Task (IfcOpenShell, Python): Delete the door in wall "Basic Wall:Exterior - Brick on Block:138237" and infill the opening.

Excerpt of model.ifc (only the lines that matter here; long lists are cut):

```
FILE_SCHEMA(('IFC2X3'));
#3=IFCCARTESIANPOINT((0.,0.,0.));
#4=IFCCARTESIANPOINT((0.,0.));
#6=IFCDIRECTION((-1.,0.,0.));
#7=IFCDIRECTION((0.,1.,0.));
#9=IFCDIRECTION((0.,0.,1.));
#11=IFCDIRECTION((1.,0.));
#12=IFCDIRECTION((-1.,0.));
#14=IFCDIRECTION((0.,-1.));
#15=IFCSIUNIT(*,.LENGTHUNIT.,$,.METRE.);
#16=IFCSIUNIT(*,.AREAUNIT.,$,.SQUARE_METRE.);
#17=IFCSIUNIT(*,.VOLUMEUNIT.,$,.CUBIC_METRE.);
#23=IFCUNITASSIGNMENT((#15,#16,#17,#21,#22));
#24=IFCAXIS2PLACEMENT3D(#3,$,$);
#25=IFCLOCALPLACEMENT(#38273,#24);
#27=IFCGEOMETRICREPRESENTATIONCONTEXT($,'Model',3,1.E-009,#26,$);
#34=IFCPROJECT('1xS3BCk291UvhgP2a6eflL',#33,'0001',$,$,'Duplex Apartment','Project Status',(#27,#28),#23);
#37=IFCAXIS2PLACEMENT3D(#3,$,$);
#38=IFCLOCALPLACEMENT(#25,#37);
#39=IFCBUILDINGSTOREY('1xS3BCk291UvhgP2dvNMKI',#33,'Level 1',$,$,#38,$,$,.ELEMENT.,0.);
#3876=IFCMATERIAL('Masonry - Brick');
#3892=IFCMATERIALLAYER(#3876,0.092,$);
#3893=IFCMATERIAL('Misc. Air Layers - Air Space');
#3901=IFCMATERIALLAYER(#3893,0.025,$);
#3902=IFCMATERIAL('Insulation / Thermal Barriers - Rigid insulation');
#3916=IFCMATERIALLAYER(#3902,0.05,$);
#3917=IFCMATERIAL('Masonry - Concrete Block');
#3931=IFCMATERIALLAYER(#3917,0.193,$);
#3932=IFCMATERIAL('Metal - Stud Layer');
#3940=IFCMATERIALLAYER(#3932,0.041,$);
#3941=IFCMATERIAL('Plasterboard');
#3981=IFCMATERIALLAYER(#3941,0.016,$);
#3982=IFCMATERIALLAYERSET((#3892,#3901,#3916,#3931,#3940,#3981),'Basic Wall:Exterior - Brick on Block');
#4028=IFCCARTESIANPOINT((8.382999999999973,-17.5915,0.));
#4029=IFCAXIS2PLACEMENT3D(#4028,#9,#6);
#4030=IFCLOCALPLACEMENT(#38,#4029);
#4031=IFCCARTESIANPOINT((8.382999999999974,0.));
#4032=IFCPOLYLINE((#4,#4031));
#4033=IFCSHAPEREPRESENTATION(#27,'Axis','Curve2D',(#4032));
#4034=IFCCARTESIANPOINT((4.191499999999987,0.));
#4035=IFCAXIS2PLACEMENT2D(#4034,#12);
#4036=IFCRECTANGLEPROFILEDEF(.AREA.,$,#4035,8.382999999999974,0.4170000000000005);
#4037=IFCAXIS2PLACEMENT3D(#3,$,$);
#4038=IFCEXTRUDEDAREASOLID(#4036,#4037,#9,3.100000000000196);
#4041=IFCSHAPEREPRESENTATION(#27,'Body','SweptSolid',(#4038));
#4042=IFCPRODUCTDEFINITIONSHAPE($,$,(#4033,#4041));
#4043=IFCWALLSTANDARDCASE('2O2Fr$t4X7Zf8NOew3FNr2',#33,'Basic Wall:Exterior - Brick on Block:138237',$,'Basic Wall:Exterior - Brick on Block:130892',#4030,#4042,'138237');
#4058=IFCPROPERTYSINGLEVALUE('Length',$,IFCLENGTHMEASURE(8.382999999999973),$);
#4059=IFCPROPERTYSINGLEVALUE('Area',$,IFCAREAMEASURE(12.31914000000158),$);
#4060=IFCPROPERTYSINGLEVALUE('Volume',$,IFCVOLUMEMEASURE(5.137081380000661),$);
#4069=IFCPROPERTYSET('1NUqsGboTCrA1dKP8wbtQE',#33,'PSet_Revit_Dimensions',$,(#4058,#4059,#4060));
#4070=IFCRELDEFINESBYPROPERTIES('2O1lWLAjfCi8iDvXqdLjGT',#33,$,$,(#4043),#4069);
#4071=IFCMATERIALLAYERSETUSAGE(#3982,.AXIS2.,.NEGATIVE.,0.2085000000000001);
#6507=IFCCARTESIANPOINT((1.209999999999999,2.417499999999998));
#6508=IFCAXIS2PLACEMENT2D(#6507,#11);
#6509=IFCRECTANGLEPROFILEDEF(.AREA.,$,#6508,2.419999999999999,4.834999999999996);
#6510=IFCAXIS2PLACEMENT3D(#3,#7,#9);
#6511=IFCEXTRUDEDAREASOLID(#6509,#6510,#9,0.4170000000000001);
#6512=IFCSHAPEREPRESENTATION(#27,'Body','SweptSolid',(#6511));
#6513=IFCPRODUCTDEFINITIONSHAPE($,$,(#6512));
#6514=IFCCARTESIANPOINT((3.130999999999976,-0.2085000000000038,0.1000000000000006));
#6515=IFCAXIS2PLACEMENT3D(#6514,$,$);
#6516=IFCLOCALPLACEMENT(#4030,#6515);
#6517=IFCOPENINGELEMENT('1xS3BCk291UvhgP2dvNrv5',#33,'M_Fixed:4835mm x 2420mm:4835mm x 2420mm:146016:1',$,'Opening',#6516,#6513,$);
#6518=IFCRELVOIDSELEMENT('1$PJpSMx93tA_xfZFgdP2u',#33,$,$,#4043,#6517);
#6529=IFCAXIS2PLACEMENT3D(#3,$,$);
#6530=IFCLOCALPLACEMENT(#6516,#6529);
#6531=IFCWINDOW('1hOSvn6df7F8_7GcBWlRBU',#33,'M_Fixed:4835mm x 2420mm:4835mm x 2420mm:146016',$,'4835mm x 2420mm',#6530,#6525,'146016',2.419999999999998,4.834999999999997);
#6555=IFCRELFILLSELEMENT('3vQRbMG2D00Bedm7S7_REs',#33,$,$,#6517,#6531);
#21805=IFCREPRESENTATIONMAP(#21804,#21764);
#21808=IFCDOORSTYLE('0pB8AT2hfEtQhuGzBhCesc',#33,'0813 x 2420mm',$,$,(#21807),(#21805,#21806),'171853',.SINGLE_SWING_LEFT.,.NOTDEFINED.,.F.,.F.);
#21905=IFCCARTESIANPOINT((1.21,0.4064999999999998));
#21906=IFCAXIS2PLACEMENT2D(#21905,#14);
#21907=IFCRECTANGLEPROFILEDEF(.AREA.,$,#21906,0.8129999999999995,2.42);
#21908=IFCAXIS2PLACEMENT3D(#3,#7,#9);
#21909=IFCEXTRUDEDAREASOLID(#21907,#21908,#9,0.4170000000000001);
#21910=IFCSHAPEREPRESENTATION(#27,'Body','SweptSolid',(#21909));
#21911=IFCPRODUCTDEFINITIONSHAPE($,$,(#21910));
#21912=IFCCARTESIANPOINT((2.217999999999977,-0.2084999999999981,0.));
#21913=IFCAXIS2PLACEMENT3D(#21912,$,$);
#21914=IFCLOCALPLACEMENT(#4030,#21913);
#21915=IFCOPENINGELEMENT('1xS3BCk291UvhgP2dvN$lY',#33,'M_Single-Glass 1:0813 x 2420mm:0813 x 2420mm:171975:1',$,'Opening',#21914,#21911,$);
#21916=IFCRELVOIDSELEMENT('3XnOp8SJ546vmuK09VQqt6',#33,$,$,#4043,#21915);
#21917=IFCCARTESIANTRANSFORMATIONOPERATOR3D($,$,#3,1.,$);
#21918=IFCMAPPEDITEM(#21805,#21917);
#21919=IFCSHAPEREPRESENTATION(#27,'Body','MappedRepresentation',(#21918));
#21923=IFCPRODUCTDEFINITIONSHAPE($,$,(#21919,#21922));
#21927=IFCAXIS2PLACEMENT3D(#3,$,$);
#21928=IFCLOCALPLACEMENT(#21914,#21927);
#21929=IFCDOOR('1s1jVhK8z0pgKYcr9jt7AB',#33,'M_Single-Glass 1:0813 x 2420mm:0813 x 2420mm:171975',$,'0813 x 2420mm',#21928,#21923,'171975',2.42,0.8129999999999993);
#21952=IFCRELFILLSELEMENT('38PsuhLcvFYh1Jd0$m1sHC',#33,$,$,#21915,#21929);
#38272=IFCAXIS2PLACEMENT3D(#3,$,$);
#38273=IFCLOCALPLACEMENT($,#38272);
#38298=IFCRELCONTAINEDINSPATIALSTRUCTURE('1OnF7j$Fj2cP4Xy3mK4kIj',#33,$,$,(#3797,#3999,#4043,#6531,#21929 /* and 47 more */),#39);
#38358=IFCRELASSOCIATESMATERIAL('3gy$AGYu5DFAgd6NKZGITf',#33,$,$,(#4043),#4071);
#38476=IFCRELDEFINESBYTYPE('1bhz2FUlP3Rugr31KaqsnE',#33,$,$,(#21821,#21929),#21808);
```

```python
import ifcopenshell
import ifcopenshell.api.feature
import ifcopenshell.api.pset
import ifcopenshell.api.root
import ifcopenshell.geom
import ifcopenshell.util.element
import ifcopenshell.util.shape
import ifcopenshell.util.unit

model = ifcopenshell.open("model.ifc")
area_scale = ifcopenshell.util.unit.calculate_unit_scale(model, "AREAUNIT")
volume_scale = ifcopenshell.util.unit.calculate_unit_scale(model, "VOLUMEUNIT")
settings = ifcopenshell.geom.settings()


def volume(element):
    """Net volume in cubic metres, openings subtracted."""
    shape = ifcopenshell.geom.create_shape(settings, element)
    return ifcopenshell.util.shape.get_volume(shape.geometry)


door = model.by_guid("1s1jVhK8z0pgKYcr9jt7AB")
opening = door.FillsVoids[0].RelatingOpeningElement
wall = opening.VoidsElements[0].RelatingBuildingElement
before = volume(wall)

ifcopenshell.api.root.remove_product(model, product=door)
ifcopenshell.api.feature.remove_feature(model, feature=opening)

after = volume(wall)
thickness = 0.417  # wall thickness in metres

# Update the wall's stored quantities.
pset = model.by_id(ifcopenshell.util.element.get_pset(wall, "PSet_Revit_Dimensions", should_inherit=False)["id"])
ifcopenshell.api.pset.edit_pset(model, pset=pset, properties={
    "Area": model.create_entity("IfcAreaMeasure", after / thickness / area_scale),
    "Volume": model.create_entity("IfcVolumeMeasure", after / volume_scale),
})

print(f"wall volume {before:.3f} -> {after:.3f} m3")

model.write("model_rev.ifc")
```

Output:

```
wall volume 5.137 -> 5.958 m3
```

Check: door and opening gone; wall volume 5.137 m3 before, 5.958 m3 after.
